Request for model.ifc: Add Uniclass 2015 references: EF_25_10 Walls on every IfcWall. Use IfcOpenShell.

First a look at what the model holds.

```python
import ifcopenshell

model = ifcopenshell.open("model.ifc")
print(model.schema)
print("classifications:", [c.Name for c in model.by_type("IfcClassification")])
for ifc_class in ("IfcDoor", "IfcRoof", "IfcStair", "IfcWall", "IfcWindow"):
    print(ifc_class, len(model.by_type(ifc_class)))
```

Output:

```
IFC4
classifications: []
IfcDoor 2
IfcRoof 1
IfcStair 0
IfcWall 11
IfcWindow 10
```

```python
import ifcopenshell
import ifcopenshell.api.classification

model = ifcopenshell.open("model.ifc")

system = ifcopenshell.api.classification.add_classification(model, classification="Uniclass 2015")

codes = {
    "IfcWall": ("EF_25_10", "Walls"),
}
for ifc_class, (code, name) in codes.items():
    products = model.by_type(ifc_class)
    ifcopenshell.api.classification.add_reference(
        model, products=products, classification=system, identification=code, name=name
    )
    print(code, len(products))

model.write("model_edited.ifc")
```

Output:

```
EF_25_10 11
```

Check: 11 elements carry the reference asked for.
